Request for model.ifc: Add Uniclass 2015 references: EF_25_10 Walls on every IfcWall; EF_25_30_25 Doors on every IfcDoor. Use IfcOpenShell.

First a look at what the model holds.

```python
import ifcopenshell

model = ifcopenshell.open("model.ifc")
print(model.schema)
print("classifications:", [c.Name for c in model.by_type("IfcClassification")])
for ifc_class in ("IfcDoor", "IfcRoof", "IfcStair", "IfcWall", "IfcWindow"):
    print(ifc_class, len(model.by_type(ifc_class)))
```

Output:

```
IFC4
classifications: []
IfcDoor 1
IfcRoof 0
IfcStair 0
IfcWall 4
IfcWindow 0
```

```python
import ifcopenshell
import ifcopenshell.api.classification

model = ifcopenshell.open("model.ifc")

system = ifcopenshell.api.classification.add_classification(model, classification="Uniclass 2015")

codes = {
    "IfcWall": ("EF_25_10", "Walls"),
    "IfcDoor": ("EF_25_30_25", "Doors"),
}
for ifc_class, (code, name) in codes.items():
    products = model.by_type(ifc_class)
    ifcopenshell.api.classification.add_reference(
        model, products=products, classification=system, identification=code, name=name
    )
    print(code, len(products))

model.write("model_rev.ifc")
```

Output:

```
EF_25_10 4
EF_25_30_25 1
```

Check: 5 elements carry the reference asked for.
